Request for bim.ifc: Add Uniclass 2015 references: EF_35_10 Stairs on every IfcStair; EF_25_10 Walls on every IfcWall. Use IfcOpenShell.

First a look at what the model holds.

```python
import ifcopenshell

model = ifcopenshell.open("bim.ifc")
print(model.schema)
print("classifications:", [c.Name for c in model.by_type("IfcClassification")])
for ifc_class in ("IfcDoor", "IfcRoof", "IfcStair", "IfcWall", "IfcWindow"):
    print(ifc_class, len(model.by_type(ifc_class)))
```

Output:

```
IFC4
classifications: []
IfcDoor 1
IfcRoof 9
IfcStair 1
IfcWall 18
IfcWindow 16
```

```python
import ifcopenshell
import ifcopenshell.api.classification

model = ifcopenshell.open("bim.ifc")

system = ifcopenshell.api.classification.add_classification(model, classification="Uniclass 2015")

codes = {
    "IfcStair": ("EF_35_10", "Stairs"),
    "IfcWall": ("EF_25_10", "Walls"),
}
for ifc_class, (code, name) in codes.items():
    products = model.by_type(ifc_class)
    ifcopenshell.api.classification.add_reference(
        model, products=products, classification=system, identification=code, name=name
    )
    print(code, len(products))

model.write("bim-out.ifc")
```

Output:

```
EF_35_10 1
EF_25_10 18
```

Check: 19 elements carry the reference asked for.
